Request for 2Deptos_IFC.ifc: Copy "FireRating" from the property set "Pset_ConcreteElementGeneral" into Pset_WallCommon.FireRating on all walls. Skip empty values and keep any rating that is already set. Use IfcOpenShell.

First a look at what the model holds.

```python
import ifcopenshell
import ifcopenshell.util.element

model = ifcopenshell.open("2Deptos_IFC.ifc")
print(model.schema)
walls = model.by_type("IfcWall")
print(len(walls), "walls")
for e in walls[:8]:
    source = ifcopenshell.util.element.get_pset(e, "Pset_ConcreteElementGeneral", "FireRating")
    target = ifcopenshell.util.element.get_pset(e, "Pset_WallCommon", "FireRating")
    print(e.id(), repr(source), repr(target), sep=" | ")
```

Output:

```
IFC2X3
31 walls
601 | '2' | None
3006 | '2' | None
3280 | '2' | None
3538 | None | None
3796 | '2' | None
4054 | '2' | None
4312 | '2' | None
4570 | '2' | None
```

```python
import ifcopenshell
import ifcopenshell.api.pset
import ifcopenshell.util.element

model = ifcopenshell.open("2Deptos_IFC.ifc")

count = 0
for e in model.by_type("IfcWall"):
    value = ifcopenshell.util.element.get_pset(e, "Pset_ConcreteElementGeneral", "FireRating")
    current = ifcopenshell.util.element.get_pset(e, "Pset_WallCommon", "FireRating")
    if not value or not value.strip() or current:
        continue
    # add_pset returns the element's existing set when there is one.
    pset = ifcopenshell.api.pset.add_pset(model, product=e, name="Pset_WallCommon")
    ifcopenshell.api.pset.edit_pset(model, pset=pset, properties={"FireRating": value})
    count += 1

print(count, "walls updated")

model.write("2Deptos_IFC_updated.ifc")
```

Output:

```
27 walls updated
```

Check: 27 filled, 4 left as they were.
